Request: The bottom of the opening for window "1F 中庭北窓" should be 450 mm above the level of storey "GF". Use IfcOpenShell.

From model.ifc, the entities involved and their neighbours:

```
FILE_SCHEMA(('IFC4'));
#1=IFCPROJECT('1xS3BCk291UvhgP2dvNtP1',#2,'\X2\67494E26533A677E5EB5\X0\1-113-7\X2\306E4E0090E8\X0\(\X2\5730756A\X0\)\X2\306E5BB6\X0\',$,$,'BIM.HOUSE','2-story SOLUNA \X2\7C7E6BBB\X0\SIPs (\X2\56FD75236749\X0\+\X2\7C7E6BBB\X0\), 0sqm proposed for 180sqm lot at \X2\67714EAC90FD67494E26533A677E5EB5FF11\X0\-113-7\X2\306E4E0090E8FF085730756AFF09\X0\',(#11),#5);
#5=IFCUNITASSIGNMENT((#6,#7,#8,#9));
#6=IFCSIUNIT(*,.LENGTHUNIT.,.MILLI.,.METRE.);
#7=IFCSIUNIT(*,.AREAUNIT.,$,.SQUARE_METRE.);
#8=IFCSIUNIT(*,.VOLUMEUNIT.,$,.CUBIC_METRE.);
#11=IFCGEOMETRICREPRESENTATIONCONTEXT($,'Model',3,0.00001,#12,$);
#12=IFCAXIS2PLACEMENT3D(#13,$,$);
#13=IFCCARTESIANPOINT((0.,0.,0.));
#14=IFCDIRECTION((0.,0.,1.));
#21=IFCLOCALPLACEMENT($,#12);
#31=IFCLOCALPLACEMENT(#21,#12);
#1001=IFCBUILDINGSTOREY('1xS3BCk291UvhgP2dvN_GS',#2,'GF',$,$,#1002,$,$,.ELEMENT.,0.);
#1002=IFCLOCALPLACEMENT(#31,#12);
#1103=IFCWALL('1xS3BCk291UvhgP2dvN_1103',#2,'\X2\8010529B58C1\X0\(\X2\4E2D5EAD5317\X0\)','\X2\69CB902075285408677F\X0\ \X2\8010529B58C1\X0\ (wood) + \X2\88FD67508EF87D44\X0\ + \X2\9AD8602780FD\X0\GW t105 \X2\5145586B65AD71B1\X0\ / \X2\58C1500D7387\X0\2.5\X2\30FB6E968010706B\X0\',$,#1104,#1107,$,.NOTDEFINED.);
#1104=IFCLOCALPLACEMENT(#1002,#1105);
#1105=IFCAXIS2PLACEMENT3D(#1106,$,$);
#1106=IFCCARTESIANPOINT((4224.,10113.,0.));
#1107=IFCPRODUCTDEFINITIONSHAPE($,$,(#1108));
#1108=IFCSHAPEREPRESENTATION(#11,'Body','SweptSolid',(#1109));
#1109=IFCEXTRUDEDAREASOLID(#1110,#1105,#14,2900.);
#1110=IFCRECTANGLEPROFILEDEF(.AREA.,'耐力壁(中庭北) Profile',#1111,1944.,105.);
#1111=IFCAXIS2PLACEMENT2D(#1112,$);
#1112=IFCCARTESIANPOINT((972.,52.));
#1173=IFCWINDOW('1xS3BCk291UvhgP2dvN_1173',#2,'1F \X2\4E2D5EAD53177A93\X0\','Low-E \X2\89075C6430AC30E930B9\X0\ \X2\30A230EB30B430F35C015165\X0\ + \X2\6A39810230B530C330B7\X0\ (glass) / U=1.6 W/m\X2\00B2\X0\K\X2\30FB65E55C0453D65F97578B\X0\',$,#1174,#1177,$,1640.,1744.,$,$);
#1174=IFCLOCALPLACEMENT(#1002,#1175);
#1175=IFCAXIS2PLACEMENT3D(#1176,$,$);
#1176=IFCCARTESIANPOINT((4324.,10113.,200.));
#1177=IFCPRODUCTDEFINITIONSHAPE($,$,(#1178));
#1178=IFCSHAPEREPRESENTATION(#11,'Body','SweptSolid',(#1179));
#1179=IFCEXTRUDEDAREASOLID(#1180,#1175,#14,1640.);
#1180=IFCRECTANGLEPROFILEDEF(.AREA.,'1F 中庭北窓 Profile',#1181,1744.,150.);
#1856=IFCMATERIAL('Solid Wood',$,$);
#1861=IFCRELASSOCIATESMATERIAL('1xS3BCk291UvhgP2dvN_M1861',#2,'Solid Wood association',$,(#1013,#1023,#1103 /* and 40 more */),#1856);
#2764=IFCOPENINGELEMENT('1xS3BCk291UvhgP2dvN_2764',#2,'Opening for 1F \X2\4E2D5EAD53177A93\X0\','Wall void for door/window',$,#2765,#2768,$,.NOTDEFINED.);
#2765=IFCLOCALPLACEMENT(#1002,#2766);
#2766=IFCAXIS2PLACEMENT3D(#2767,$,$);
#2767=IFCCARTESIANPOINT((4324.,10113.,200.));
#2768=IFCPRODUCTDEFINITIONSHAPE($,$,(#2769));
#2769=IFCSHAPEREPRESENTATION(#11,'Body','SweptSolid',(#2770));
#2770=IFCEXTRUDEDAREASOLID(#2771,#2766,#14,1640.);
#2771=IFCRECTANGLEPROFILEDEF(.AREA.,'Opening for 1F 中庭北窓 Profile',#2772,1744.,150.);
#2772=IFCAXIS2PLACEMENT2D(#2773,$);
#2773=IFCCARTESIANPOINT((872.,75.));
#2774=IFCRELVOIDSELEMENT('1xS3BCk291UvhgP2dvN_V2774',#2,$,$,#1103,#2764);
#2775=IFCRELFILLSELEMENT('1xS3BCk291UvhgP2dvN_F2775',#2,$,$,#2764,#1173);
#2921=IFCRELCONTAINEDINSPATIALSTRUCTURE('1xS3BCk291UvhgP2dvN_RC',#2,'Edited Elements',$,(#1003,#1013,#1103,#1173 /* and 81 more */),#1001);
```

```python
import numpy as np
import ifcopenshell
import ifcopenshell.api.geometry
import ifcopenshell.geom
import ifcopenshell.util.element
import ifcopenshell.util.placement
import ifcopenshell.util.shape
import ifcopenshell.util.unit

model = ifcopenshell.open("model.ifc")
unit_scale = ifcopenshell.util.unit.calculate_unit_scale(model)

window = model.by_guid("1xS3BCk291UvhgP2dvN_1173")
opening = window.FillsVoids[0].RelatingOpeningElement
storey = ifcopenshell.util.element.get_container(window, ifc_class="IfcBuildingStorey")
level = ifcopenshell.util.placement.get_local_placement(storey.ObjectPlacement)[2, 3]

# The opening's origin need not be at the sill, so measure its lowest point.
shape = ifcopenshell.geom.create_shape(ifcopenshell.geom.settings(), opening)
bottom = ifcopenshell.util.shape.get_shape_bottom_elevation(shape, shape.geometry) / unit_scale
dz = level + 450.0 - bottom

shift = np.array([0.0, 0.0, dz])
# The window is not placed relative to its opening, so move both.
for product in (opening, window):
    matrix = ifcopenshell.util.placement.get_local_placement(product.ObjectPlacement)
    matrix[:3, 3] += shift
    ifcopenshell.api.geometry.edit_object_placement(model, product=product, matrix=matrix, is_si=False)

print(f"moved by {dz * unit_scale:+.3f} m")

model.write("model_v2.ifc")
```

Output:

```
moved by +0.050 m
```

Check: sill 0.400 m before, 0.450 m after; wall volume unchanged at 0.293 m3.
